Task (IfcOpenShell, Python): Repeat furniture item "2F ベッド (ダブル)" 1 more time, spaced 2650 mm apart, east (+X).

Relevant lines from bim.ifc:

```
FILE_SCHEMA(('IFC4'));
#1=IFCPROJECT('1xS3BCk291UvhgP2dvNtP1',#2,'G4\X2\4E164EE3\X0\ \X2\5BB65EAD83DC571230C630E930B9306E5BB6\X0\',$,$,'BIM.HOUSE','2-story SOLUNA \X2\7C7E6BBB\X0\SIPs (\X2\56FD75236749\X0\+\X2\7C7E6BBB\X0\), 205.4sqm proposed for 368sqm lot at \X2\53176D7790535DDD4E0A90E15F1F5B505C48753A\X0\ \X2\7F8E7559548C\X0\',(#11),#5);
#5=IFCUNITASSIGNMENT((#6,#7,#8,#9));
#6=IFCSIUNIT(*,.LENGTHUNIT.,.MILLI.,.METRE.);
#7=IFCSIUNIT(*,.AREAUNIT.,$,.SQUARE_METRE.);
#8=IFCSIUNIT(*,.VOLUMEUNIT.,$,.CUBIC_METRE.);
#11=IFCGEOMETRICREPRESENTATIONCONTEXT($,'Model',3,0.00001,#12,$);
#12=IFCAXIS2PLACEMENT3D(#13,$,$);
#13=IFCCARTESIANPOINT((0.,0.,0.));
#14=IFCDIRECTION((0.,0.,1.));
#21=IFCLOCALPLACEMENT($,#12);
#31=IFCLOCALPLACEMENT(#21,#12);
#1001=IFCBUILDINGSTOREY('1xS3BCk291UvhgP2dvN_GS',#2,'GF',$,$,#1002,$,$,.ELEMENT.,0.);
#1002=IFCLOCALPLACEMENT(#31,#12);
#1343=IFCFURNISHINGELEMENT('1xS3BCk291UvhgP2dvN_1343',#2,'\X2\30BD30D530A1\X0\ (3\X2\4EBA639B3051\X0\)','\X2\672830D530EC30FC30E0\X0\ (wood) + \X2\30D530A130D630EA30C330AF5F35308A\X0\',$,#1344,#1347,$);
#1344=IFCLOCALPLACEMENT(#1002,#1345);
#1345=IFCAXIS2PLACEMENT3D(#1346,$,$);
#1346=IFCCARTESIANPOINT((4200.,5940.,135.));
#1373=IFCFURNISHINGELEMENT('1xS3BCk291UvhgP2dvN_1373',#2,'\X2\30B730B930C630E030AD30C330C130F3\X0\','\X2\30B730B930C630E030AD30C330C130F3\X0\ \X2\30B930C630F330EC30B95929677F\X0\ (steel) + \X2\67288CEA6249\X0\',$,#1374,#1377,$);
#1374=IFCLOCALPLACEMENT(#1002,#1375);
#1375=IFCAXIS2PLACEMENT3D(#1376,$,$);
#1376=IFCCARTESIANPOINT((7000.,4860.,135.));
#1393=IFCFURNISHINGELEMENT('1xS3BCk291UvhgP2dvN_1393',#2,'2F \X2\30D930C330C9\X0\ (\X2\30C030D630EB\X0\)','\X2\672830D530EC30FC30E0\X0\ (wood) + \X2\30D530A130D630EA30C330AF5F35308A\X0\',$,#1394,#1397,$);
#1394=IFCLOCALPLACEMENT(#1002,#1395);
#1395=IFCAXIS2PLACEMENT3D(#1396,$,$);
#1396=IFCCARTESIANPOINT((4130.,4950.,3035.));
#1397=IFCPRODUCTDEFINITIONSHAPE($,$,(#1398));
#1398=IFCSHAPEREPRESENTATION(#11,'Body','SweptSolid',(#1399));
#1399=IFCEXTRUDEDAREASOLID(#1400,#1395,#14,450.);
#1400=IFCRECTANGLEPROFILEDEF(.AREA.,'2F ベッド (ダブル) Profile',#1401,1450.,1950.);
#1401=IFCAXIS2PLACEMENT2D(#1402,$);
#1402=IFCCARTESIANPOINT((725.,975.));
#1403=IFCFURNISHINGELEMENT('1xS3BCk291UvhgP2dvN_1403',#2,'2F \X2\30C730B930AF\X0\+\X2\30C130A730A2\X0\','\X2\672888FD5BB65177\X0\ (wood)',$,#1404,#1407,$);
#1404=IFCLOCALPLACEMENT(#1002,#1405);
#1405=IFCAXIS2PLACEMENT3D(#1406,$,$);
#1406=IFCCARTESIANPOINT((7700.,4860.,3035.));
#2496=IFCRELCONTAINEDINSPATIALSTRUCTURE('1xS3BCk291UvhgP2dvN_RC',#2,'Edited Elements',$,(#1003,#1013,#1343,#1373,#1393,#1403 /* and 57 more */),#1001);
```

```python
import numpy as np
import ifcopenshell
import ifcopenshell.api.geometry
import ifcopenshell.api.root
import ifcopenshell.util.element
import ifcopenshell.util.placement
import ifcopenshell.util.unit

model = ifcopenshell.open("bim.ifc")
unit_scale = ifcopenshell.util.unit.calculate_unit_scale(model)


def reuse_history(source, copy):
    """copy_class also copies each property set's owner history, people and application; keep the originals."""
    for rel in copy.IsDefinedBy:
        if rel.is_a("IfcRelDefinesByProperties") and (history := rel.RelatingPropertyDefinition.OwnerHistory):
            rel.RelatingPropertyDefinition.OwnerHistory = source.OwnerHistory
            ifcopenshell.util.element.remove_deep2(model, history)


source = model.by_guid("1xS3BCk291UvhgP2dvN_1393")
base = ifcopenshell.util.placement.get_local_placement(source.ObjectPlacement)
step = np.array([1.0, 0.0, 0.0]) * 2.65 / unit_scale

for i in range(1, 2):
    copy = ifcopenshell.api.root.copy_class(model, product=source)
    copy.Representation = ifcopenshell.util.element.copy_deep(
        model, source.Representation, exclude=["IfcGeometricRepresentationContext", "IfcRepresentationMap"]
    )
    reuse_history(source, copy)
    matrix = base.copy()
    matrix[:3, 3] += i * step
    print("added at", matrix[:3, 3].round(3) + 0.0)
    ifcopenshell.api.geometry.edit_object_placement(model, product=copy, matrix=matrix, is_si=False)

model.write("bim-out.ifc")
```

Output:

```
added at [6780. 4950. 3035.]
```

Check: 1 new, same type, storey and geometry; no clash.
